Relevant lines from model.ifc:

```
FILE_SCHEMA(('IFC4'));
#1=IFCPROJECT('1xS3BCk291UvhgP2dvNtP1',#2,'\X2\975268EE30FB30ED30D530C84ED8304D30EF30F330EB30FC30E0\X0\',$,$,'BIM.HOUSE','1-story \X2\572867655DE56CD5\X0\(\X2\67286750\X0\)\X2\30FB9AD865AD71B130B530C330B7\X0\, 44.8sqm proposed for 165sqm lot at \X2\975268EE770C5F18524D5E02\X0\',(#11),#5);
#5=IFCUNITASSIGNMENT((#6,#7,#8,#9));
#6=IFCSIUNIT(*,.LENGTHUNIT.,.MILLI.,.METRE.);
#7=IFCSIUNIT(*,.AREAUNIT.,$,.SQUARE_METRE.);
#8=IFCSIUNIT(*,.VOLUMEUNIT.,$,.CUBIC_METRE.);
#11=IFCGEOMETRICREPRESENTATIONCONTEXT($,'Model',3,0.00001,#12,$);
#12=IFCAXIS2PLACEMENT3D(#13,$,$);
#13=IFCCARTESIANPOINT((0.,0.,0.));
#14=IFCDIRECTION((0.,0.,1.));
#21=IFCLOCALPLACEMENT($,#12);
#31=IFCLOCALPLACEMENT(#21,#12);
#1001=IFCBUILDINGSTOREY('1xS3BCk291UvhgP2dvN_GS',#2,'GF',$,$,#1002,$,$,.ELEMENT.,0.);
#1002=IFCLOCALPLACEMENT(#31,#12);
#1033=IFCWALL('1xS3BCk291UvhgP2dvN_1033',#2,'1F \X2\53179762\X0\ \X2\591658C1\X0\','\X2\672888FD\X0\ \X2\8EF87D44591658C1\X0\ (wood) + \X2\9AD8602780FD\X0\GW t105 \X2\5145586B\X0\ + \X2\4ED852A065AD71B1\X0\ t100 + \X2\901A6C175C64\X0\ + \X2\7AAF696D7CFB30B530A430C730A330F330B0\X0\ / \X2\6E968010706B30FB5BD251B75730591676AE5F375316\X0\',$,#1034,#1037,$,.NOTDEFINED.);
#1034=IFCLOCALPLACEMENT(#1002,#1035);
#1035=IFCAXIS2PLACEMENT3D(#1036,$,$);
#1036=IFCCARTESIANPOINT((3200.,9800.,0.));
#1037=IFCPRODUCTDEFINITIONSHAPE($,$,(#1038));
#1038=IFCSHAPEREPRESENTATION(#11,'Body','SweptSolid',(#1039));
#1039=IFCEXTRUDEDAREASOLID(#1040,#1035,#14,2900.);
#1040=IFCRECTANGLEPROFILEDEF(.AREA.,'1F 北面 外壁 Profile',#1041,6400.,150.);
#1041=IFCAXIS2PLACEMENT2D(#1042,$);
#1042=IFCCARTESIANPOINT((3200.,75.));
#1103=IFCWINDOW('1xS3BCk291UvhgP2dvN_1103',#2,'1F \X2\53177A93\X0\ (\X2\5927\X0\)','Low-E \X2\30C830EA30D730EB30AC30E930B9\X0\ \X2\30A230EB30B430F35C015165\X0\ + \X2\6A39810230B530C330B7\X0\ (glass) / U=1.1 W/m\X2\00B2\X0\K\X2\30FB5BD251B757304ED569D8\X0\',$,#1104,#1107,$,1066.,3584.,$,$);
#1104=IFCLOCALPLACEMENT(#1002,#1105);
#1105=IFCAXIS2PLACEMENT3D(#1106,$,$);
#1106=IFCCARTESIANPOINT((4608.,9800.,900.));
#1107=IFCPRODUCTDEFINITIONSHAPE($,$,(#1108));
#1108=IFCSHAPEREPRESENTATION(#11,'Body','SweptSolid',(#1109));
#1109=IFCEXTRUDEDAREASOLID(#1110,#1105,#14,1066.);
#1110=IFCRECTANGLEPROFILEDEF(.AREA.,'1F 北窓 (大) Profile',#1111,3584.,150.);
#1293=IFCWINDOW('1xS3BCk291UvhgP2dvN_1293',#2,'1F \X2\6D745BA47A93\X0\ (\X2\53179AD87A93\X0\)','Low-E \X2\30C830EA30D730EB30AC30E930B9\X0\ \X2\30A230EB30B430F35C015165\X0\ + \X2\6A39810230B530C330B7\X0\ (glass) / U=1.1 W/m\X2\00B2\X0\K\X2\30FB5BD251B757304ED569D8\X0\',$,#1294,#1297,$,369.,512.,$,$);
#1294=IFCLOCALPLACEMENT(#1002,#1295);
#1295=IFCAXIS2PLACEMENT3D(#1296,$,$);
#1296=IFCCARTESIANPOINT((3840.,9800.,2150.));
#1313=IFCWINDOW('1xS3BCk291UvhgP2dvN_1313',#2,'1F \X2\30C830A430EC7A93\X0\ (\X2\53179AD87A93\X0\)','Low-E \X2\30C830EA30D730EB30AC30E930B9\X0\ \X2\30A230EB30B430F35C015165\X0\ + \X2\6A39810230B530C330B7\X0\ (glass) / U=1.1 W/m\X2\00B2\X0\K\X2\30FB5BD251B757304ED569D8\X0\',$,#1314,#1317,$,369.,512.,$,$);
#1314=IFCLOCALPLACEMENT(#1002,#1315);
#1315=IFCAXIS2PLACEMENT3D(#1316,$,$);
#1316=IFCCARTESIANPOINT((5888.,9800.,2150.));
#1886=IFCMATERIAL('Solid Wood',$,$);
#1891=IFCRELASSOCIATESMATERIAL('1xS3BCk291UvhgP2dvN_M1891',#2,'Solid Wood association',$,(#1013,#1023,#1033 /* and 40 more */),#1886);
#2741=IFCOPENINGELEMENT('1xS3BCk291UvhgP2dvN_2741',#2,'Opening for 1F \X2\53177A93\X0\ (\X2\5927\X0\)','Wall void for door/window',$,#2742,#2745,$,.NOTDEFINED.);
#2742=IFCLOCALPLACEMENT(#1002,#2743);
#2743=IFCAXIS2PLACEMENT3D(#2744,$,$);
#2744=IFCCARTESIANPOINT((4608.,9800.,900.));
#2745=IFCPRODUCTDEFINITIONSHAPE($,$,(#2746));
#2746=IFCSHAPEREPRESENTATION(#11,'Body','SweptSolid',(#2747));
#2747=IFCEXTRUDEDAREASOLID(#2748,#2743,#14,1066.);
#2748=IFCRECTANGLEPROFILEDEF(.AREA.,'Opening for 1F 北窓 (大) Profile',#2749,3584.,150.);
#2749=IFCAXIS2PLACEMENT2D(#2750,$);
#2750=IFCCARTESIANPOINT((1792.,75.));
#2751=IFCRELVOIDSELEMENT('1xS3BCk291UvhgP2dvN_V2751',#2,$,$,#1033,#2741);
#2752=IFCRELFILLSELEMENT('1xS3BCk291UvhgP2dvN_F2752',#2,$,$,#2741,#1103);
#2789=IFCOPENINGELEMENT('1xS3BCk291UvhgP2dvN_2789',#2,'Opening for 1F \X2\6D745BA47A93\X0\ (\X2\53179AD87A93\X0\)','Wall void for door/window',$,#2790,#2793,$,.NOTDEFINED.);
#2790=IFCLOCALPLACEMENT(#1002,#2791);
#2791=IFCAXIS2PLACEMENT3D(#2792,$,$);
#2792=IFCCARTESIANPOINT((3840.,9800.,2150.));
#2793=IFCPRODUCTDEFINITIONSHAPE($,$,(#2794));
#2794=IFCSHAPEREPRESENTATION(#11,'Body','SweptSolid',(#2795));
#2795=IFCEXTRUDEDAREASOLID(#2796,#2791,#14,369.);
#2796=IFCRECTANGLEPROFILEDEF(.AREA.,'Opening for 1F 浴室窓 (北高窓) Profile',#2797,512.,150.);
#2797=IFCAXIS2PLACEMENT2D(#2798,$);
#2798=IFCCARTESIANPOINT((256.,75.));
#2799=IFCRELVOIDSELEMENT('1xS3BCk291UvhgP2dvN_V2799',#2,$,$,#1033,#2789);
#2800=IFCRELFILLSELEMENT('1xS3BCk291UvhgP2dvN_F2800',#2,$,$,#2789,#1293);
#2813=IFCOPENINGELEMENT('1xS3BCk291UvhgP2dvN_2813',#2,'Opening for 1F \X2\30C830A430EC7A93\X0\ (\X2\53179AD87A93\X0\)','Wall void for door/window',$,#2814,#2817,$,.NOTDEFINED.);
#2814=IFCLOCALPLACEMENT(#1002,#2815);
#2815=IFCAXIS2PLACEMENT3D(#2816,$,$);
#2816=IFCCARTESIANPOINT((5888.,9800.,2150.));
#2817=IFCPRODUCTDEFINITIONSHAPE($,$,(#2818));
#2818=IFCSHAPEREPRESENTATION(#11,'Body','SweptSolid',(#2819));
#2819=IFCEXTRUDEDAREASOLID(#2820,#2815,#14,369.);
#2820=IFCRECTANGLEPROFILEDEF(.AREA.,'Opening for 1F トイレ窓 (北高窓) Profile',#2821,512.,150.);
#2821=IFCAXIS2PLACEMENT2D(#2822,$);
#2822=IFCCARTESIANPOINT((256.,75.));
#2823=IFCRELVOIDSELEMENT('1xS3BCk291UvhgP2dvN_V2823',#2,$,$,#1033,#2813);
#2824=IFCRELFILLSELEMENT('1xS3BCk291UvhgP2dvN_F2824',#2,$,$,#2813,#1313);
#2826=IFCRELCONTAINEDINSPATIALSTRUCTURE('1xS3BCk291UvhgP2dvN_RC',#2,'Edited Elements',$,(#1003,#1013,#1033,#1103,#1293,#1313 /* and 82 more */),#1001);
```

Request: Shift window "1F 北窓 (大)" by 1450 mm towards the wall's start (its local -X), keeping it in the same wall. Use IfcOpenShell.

```python
import ifcopenshell
import ifcopenshell.api.geometry
import ifcopenshell.util.placement

model = ifcopenshell.open("model.ifc")

window = model.by_guid("1xS3BCk291UvhgP2dvN_1103")
opening = window.FillsVoids[0].RelatingOpeningElement
wall = opening.VoidsElements[0].RelatingBuildingElement

wall_matrix = ifcopenshell.util.placement.get_local_placement(wall.ObjectPlacement)
shift = wall_matrix[:3, 0] * -1450.0
before = ifcopenshell.util.placement.get_local_placement(window.ObjectPlacement)[:3, 3].copy()

# The window is not placed relative to its opening, so move both.
for product in (opening, window):
    matrix = ifcopenshell.util.placement.get_local_placement(product.ObjectPlacement)
    matrix[:3, 3] += shift
    ifcopenshell.api.geometry.edit_object_placement(model, product=product, matrix=matrix, is_si=False)

after = ifcopenshell.util.placement.get_local_placement(window.ObjectPlacement)[:3, 3]
print("window moved by", (after - before).round(3) + 0.0)

model.write("model_v2.ifc")
```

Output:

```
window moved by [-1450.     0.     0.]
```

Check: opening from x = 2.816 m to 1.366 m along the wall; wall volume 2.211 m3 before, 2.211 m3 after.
